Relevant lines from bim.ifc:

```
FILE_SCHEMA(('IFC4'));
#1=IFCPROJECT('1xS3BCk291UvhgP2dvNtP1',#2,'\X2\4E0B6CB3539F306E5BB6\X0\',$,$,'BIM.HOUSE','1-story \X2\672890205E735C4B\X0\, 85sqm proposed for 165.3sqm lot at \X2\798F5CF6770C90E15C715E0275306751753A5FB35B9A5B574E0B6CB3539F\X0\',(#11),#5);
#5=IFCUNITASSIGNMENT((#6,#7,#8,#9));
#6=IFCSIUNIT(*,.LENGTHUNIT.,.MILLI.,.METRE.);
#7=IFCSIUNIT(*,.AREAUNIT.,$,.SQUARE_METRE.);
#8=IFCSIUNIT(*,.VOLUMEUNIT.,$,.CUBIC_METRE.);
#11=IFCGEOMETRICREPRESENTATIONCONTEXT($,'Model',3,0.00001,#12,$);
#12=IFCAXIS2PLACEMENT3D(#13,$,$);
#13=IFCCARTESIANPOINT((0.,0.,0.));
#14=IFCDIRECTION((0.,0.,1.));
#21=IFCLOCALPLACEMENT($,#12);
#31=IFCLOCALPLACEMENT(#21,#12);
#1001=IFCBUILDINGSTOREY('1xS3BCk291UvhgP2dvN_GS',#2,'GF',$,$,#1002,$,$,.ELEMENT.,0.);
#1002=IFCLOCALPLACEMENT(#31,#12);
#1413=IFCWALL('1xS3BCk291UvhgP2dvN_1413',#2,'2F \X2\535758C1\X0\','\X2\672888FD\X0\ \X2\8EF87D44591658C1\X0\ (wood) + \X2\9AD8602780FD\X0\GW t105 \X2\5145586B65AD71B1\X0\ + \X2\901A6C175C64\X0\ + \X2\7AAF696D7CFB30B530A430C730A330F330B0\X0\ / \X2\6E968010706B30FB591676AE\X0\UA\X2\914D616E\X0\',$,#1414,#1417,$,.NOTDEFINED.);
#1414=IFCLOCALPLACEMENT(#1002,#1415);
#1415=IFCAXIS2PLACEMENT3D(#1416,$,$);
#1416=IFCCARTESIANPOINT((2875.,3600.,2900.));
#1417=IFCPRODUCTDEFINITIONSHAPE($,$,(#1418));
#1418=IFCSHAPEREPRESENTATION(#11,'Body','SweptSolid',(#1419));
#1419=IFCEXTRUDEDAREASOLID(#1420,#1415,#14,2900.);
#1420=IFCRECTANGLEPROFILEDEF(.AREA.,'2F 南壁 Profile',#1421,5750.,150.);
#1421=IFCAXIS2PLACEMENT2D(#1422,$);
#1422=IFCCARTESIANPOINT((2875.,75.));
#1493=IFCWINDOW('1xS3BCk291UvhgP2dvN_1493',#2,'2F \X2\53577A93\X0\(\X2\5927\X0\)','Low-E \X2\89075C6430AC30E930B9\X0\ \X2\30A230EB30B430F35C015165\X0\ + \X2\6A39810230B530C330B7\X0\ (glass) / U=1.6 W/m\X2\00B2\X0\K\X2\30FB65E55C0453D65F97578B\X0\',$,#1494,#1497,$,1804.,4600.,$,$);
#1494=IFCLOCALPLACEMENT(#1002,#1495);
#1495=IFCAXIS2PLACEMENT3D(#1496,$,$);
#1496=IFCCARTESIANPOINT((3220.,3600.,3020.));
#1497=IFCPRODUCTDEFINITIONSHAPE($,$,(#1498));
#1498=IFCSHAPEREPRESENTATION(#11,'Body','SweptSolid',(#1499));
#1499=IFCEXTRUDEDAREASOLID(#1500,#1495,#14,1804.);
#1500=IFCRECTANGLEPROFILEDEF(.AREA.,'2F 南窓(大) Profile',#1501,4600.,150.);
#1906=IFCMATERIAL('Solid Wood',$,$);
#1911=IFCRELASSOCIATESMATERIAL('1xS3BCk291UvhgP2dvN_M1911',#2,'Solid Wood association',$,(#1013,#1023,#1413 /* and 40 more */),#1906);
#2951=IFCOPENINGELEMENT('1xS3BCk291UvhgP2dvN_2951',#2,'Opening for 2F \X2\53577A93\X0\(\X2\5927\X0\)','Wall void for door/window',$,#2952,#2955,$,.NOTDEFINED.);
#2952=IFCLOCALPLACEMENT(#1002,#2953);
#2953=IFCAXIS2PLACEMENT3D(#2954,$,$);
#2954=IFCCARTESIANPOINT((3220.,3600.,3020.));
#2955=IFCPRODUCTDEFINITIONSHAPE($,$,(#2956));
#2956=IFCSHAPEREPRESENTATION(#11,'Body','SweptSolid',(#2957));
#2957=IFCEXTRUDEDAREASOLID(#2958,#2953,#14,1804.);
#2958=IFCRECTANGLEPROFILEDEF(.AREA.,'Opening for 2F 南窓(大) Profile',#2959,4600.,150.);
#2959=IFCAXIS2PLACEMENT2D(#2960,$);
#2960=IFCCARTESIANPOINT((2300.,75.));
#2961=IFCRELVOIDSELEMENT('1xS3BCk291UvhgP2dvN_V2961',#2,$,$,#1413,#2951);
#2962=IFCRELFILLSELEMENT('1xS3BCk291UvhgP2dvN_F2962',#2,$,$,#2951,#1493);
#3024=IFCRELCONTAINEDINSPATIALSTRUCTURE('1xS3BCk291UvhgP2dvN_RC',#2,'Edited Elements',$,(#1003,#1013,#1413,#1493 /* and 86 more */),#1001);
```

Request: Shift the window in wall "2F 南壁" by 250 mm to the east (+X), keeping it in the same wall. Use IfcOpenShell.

```python
import ifcopenshell
import ifcopenshell.api.geometry
import ifcopenshell.util.placement

model = ifcopenshell.open("bim.ifc")

window = model.by_id(1493)
opening = window.FillsVoids[0].RelatingOpeningElement
wall = opening.VoidsElements[0].RelatingBuildingElement

wall_matrix = ifcopenshell.util.placement.get_local_placement(wall.ObjectPlacement)
shift = wall_matrix[:3, 0] * 250.0
before = ifcopenshell.util.placement.get_local_placement(window.ObjectPlacement)[:3, 3].copy()

# The window is not placed relative to its opening, so move both.
for product in (opening, window):
    matrix = ifcopenshell.util.placement.get_local_placement(product.ObjectPlacement)
    matrix[:3, 3] += shift
    ifcopenshell.api.geometry.edit_object_placement(model, product=product, matrix=matrix, is_si=False)

after = ifcopenshell.util.placement.get_local_placement(window.ObjectPlacement)[:3, 3]
print("window moved by", (after - before).round(3) + 0.0)

model.write("bim_v2.ifc")
```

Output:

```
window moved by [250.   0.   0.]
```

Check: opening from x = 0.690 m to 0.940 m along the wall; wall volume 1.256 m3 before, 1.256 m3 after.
